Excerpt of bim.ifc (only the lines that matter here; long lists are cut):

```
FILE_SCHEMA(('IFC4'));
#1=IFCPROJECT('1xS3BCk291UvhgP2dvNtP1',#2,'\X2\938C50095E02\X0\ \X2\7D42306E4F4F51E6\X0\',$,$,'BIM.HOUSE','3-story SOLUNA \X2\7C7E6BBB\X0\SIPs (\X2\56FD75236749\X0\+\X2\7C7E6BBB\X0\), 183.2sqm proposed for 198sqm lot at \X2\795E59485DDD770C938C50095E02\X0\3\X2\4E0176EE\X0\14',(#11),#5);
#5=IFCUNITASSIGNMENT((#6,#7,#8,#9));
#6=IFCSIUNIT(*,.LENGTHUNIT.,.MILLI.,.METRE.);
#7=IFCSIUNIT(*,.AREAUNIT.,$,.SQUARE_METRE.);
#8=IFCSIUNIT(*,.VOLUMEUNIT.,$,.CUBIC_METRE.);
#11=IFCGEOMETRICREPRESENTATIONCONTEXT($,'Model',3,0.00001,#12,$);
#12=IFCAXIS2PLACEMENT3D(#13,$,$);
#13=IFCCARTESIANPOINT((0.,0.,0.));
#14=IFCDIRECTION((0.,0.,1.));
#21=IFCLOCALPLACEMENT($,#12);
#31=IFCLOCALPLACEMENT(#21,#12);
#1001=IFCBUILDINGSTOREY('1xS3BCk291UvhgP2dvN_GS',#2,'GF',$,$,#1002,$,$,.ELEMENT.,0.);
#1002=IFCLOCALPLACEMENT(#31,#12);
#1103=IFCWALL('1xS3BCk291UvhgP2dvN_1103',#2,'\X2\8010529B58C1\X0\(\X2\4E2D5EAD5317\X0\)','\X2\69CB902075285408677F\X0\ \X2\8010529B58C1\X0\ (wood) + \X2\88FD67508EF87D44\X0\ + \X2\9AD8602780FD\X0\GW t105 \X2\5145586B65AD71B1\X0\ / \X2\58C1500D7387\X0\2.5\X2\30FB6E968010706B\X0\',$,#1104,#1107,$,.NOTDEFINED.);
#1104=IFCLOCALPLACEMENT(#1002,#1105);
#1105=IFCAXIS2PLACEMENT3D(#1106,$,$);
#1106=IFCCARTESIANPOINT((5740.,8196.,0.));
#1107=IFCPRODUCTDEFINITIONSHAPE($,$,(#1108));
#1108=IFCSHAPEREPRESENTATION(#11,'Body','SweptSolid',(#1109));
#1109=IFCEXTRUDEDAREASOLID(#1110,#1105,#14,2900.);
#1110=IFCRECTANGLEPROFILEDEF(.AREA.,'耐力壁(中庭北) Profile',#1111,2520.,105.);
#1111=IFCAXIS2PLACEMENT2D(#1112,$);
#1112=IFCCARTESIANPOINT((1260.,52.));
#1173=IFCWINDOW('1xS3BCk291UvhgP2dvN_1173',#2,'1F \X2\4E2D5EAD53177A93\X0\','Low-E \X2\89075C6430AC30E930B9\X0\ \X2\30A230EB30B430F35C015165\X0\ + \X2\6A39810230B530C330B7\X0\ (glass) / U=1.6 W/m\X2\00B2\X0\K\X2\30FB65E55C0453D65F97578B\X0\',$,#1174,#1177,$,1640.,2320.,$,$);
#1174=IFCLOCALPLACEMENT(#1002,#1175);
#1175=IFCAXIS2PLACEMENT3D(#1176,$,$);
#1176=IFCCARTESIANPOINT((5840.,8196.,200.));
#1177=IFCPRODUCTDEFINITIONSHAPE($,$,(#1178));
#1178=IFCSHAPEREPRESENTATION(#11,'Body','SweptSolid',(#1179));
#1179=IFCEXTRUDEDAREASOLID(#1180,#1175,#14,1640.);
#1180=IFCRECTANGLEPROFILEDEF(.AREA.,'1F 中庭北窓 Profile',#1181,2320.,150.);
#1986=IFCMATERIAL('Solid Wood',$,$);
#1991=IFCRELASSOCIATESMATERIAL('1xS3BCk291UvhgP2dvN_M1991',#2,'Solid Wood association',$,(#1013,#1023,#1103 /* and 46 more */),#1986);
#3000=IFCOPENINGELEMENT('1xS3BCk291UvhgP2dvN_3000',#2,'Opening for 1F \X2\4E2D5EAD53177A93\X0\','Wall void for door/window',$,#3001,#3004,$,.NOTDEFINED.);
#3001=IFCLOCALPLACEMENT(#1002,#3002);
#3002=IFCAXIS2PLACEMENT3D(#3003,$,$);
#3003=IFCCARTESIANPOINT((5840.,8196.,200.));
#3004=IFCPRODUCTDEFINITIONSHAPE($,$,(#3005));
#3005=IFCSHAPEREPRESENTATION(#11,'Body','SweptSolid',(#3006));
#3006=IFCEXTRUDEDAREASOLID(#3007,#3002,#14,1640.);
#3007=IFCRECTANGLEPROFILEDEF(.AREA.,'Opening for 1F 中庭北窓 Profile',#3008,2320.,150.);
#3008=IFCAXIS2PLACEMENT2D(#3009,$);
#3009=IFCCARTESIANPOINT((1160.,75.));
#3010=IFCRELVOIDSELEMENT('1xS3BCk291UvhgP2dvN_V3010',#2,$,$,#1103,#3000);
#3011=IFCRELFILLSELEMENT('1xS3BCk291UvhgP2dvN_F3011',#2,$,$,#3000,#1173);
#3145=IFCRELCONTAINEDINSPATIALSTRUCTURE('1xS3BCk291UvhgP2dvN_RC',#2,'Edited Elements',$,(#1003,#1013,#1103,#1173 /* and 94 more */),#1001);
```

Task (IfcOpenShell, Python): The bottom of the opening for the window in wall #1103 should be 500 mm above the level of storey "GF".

```python
import numpy as np
import ifcopenshell
import ifcopenshell.api.geometry
import ifcopenshell.geom
import ifcopenshell.util.element
import ifcopenshell.util.placement
import ifcopenshell.util.shape
import ifcopenshell.util.unit

model = ifcopenshell.open("bim.ifc")
unit_scale = ifcopenshell.util.unit.calculate_unit_scale(model)

window = model.by_guid("1xS3BCk291UvhgP2dvN_1173")
opening = window.FillsVoids[0].RelatingOpeningElement
storey = ifcopenshell.util.element.get_container(window, ifc_class="IfcBuildingStorey")
level = ifcopenshell.util.placement.get_local_placement(storey.ObjectPlacement)[2, 3]

# The opening's origin need not be at the sill, so measure its lowest point.
shape = ifcopenshell.geom.create_shape(ifcopenshell.geom.settings(), opening)
bottom = ifcopenshell.util.shape.get_shape_bottom_elevation(shape, shape.geometry) / unit_scale
dz = level + 0.5 / unit_scale - bottom

shift = np.array([0.0, 0.0, dz])
# The window is not placed relative to its opening, so move both.
for product in (opening, window):
    matrix = ifcopenshell.util.placement.get_local_placement(product.ObjectPlacement)
    matrix[:3, 3] += shift
    ifcopenshell.api.geometry.edit_object_placement(model, product=product, matrix=matrix, is_si=False)

print(f"moved by {dz * unit_scale:+.3f} m")

model.write("bim_v2.ifc")
```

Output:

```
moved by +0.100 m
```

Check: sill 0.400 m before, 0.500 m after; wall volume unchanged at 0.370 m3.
